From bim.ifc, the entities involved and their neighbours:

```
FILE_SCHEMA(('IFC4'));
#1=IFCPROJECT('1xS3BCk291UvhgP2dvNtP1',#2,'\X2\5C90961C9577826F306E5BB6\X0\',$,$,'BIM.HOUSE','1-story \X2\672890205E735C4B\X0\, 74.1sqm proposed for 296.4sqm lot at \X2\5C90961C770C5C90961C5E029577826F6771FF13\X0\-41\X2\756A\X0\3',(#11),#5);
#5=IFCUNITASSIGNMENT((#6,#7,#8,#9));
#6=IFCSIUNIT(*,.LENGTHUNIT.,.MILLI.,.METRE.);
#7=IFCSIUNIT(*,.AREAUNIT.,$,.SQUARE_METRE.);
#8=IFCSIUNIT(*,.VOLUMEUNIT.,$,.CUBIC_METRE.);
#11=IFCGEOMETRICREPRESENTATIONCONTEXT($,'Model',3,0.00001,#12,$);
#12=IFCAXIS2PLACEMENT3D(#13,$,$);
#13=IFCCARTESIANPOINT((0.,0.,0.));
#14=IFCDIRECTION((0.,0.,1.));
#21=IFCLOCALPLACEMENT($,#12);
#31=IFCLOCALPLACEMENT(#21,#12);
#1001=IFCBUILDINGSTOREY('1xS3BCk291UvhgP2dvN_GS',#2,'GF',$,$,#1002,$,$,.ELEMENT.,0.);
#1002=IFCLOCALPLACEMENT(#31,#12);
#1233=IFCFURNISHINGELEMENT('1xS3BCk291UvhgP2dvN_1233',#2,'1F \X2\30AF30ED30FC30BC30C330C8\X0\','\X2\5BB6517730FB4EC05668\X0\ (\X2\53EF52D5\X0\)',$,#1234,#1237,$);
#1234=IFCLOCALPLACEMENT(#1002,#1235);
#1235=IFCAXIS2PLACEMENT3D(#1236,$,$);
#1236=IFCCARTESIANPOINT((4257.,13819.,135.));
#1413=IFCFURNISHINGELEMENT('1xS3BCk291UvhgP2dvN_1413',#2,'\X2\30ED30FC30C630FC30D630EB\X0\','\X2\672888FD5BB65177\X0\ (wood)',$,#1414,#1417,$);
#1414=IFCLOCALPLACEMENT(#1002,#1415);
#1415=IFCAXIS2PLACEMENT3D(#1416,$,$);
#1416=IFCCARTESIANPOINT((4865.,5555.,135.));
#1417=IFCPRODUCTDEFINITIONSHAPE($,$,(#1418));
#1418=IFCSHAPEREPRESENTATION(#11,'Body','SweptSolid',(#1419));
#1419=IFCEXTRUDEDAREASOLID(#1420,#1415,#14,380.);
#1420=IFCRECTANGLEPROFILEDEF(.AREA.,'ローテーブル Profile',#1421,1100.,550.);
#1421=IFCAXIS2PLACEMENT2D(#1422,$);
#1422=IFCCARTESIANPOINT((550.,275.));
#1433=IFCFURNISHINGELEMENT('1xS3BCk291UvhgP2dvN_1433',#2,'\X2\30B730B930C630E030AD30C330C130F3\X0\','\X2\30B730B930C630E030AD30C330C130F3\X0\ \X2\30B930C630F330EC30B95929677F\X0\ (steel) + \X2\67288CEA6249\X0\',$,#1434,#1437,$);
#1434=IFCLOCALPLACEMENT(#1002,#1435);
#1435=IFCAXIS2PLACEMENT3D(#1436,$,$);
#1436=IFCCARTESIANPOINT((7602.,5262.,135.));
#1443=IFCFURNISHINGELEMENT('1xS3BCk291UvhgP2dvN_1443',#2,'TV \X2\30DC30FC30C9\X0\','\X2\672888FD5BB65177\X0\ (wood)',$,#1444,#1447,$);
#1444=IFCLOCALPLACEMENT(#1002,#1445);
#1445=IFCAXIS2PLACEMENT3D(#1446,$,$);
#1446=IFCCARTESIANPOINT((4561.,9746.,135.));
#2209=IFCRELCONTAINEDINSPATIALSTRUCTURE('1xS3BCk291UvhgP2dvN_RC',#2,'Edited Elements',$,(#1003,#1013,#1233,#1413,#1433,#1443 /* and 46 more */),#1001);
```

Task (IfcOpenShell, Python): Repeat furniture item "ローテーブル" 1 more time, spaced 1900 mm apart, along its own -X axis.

```python
import ifcopenshell
import ifcopenshell.api.geometry
import ifcopenshell.api.root
import ifcopenshell.util.element
import ifcopenshell.util.placement

model = ifcopenshell.open("bim.ifc")


def reuse_history(source, copy):
    """copy_class also copies each property set's owner history, people and application; keep the originals."""
    for rel in copy.IsDefinedBy:
        if rel.is_a("IfcRelDefinesByProperties") and (history := rel.RelatingPropertyDefinition.OwnerHistory):
            rel.RelatingPropertyDefinition.OwnerHistory = source.OwnerHistory
            ifcopenshell.util.element.remove_deep2(model, history)


source = model.by_id(1413)
base = ifcopenshell.util.placement.get_local_placement(source.ObjectPlacement)
step = -base[:3, 0] * 1900.0

for i in range(1, 2):
    copy = ifcopenshell.api.root.copy_class(model, product=source)
    copy.Representation = ifcopenshell.util.element.copy_deep(
        model, source.Representation, exclude=["IfcGeometricRepresentationContext", "IfcRepresentationMap"]
    )
    reuse_history(source, copy)
    matrix = base.copy()
    matrix[:3, 3] += i * step
    print("added at", matrix[:3, 3].round(3) + 0.0)
    ifcopenshell.api.geometry.edit_object_placement(model, product=copy, matrix=matrix, is_si=False)

model.write("bim_rev.ifc")
```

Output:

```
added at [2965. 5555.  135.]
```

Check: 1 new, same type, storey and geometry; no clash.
